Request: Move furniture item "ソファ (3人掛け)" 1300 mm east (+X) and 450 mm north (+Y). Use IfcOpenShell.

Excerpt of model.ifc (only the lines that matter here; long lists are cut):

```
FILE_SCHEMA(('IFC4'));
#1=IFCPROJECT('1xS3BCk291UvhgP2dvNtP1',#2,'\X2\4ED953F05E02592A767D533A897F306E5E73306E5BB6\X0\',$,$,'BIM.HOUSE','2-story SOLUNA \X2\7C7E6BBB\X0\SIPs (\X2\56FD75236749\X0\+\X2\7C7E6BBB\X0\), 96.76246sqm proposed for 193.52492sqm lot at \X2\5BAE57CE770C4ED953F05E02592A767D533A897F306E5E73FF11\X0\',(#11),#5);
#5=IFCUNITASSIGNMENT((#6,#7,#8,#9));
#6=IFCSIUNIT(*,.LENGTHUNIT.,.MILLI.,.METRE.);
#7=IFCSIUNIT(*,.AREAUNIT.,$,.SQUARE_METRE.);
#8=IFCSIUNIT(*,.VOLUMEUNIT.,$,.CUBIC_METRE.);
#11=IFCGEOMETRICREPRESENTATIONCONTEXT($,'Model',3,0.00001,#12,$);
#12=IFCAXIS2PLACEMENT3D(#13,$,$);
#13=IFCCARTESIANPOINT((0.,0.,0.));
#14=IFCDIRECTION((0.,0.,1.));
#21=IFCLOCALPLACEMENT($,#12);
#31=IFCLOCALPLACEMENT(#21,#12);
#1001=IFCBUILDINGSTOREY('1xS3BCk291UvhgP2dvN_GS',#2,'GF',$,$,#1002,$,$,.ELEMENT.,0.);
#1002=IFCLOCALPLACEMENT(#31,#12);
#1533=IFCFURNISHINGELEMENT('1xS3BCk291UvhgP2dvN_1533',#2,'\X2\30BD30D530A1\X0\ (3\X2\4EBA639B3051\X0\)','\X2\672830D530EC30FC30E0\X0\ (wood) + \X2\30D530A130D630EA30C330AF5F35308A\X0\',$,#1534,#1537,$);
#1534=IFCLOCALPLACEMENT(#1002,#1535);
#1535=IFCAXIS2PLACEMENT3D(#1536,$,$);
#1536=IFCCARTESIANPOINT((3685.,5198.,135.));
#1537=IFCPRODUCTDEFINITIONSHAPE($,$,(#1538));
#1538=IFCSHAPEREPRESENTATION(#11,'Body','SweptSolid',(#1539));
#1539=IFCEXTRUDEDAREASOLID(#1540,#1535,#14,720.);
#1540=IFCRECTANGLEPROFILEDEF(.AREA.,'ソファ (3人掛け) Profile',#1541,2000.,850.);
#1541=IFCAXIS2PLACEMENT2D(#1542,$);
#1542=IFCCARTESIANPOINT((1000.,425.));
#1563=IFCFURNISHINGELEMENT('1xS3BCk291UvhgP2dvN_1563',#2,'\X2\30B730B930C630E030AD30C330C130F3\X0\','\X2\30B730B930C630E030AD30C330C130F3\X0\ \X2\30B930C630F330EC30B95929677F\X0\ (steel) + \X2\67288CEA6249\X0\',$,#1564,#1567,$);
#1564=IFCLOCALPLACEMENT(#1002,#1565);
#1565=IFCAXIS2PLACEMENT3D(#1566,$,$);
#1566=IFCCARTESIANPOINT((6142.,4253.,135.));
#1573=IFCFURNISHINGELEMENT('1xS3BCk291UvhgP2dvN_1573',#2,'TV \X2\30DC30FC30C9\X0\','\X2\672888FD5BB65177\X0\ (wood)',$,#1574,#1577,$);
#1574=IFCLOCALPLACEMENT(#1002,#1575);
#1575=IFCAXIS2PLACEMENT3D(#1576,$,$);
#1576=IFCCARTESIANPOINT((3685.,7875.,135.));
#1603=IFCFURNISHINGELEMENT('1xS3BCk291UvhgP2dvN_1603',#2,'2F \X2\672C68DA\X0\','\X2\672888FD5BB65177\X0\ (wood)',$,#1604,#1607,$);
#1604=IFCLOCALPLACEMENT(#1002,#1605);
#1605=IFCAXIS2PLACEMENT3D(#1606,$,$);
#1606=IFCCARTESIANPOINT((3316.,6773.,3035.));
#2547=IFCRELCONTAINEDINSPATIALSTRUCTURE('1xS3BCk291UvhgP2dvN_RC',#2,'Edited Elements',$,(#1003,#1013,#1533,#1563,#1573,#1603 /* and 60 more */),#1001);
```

```python
import ifcopenshell
import ifcopenshell.api.geometry
import ifcopenshell.util.placement

model = ifcopenshell.open("model.ifc")

item = model.by_id(1533)
matrix = ifcopenshell.util.placement.get_local_placement(item.ObjectPlacement)
matrix[0, 3] += 1300.0
matrix[1, 3] += 450.0
ifcopenshell.api.geometry.edit_object_placement(model, product=item, matrix=matrix, is_si=False)

print(ifcopenshell.util.placement.get_local_placement(item.ObjectPlacement).round(3) + 0.0)

model.write("model_v2.ifc")
```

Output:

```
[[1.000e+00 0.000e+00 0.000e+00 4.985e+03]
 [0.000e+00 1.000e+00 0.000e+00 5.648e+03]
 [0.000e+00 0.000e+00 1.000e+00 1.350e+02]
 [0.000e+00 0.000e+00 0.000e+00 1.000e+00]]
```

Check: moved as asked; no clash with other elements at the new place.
